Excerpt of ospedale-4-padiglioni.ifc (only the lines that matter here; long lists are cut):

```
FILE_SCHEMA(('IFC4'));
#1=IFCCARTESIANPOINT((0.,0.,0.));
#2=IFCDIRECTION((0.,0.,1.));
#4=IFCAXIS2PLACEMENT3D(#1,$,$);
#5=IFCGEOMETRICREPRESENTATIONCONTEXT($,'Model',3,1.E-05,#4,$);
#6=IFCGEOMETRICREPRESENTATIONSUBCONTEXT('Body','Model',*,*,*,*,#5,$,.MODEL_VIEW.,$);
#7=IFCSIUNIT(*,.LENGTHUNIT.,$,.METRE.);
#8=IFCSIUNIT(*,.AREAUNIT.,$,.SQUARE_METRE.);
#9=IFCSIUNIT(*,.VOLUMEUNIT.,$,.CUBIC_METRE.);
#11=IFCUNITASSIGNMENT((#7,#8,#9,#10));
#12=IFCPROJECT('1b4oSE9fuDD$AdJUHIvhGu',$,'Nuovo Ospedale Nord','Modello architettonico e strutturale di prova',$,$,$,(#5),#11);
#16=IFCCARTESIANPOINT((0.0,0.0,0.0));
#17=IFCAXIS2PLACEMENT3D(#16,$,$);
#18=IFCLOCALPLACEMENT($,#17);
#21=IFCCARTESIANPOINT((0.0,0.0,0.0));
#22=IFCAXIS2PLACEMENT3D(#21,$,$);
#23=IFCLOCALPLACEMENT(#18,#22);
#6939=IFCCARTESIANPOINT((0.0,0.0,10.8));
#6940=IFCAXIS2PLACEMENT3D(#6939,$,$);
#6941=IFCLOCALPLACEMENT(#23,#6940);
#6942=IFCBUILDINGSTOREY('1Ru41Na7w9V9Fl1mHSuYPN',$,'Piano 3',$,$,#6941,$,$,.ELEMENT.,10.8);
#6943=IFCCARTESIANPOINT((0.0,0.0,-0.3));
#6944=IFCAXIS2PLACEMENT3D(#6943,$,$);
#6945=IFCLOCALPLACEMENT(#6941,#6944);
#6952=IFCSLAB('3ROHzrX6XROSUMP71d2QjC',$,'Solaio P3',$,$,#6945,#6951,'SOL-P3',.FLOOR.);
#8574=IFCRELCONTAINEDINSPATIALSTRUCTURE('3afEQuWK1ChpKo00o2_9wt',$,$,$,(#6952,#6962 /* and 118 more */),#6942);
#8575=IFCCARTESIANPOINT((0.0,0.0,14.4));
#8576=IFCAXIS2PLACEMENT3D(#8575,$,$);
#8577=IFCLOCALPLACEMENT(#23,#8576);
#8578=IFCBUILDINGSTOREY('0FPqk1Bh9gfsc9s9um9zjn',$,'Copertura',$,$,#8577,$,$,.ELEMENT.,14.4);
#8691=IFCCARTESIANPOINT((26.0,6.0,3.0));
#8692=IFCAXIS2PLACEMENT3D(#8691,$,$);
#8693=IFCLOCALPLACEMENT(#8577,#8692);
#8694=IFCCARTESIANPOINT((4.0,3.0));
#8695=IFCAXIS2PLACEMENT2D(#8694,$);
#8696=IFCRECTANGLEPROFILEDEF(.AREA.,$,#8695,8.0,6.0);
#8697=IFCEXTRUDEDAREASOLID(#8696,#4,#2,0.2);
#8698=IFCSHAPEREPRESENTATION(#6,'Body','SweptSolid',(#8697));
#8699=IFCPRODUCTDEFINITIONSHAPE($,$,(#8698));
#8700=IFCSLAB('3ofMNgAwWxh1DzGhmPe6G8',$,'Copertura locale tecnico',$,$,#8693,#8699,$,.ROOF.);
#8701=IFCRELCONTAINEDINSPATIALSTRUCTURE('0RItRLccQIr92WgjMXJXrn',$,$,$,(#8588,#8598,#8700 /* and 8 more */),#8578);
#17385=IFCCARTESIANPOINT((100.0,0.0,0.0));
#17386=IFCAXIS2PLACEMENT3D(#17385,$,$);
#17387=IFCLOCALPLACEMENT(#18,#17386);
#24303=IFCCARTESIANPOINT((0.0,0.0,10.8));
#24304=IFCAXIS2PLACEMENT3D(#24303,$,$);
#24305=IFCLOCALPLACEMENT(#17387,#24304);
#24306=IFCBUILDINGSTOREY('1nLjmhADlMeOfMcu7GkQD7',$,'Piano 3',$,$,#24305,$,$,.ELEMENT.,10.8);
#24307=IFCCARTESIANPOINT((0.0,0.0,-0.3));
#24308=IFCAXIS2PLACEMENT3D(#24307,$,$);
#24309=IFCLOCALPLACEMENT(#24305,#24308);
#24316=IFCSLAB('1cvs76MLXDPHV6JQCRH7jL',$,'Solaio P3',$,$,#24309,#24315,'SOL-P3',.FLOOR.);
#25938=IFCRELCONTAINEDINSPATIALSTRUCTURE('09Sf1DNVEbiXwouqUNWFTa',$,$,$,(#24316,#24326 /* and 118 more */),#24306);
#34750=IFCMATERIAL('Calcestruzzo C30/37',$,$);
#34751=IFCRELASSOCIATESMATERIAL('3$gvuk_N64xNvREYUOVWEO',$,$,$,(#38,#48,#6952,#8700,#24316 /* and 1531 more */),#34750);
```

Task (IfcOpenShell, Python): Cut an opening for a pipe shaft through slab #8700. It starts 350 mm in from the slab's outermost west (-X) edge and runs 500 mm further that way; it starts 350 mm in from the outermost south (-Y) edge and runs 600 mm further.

```python
import numpy as np
import ifcopenshell
import ifcopenshell.api.feature
import ifcopenshell.api.geometry
import ifcopenshell.api.root
import ifcopenshell.geom
import ifcopenshell.util.placement
import ifcopenshell.util.representation
import ifcopenshell.util.shape
import ifcopenshell.util.unit

model = ifcopenshell.open("ospedale-4-padiglioni.ifc")
unit_scale = ifcopenshell.util.unit.calculate_unit_scale(model)
settings = ifcopenshell.geom.settings()


def volume(element):
    """Net volume in cubic metres, openings subtracted."""
    shape = ifcopenshell.geom.create_shape(settings, element)
    return ifcopenshell.util.shape.get_volume(shape.geometry)


slab = model.by_guid("3ofMNgAwWxh1DzGhmPe6G8")
before = volume(slab)

# Extent in the slab's own axes, in metres. The edges named are its -X and -Y sides.
slab_shape = ifcopenshell.geom.create_shape(settings, slab)
vertices = ifcopenshell.util.shape.get_vertices(slab_shape.geometry)
x_min, y_min, bottom = vertices.min(axis=0)
top = vertices[:, 2].max()

opening = ifcopenshell.api.root.create_entity(model, ifc_class="IfcOpeningElement", name="Pipe shaft opening", predefined_type="OPENING")
context = ifcopenshell.util.representation.get_context(model, "Model", "Body", "MODEL_VIEW")
width, depth = 0.5, 0.6
outline = [(0.0, 0.0), (width, 0.0), (width, depth), (0.0, depth), (0.0, 0.0)]
# Overshoot both faces by 50 mm so the cut is clean.
shape = ifcopenshell.api.geometry.add_slab_representation(
    model, context=context, depth=top - bottom + 0.1, polyline=outline
)
ifcopenshell.api.geometry.assign_representation(model, product=opening, representation=shape)

matrix = ifcopenshell.util.placement.get_local_placement(slab.ObjectPlacement)
matrix[:, 3] = matrix @ np.append(np.array([x_min + 0.35, y_min + 0.35, bottom - 0.05]) / unit_scale, 1.0)
ifcopenshell.api.geometry.edit_object_placement(model, product=opening, matrix=matrix, is_si=False)
ifcopenshell.api.feature.add_feature(model, feature=opening, element=slab)

after = volume(slab)

print(f"slab volume {before:.3f} -> {after:.3f} m3")

model.write("ospedale-4-padiglioni_rev.ifc")
```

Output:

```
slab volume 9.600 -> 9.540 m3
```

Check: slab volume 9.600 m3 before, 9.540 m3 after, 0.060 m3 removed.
